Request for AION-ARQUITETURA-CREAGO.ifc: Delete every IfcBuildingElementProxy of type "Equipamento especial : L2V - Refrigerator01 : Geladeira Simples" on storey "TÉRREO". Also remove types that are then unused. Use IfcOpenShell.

First a look at what the model holds.

```python
import ifcopenshell
import ifcopenshell.util.element

model = ifcopenshell.open("AION-ARQUITETURA-CREAGO.ifc")
print(model.schema)
storey = next(s for s in model.by_type("IfcBuildingStorey") if s.Name == "TÉRREO")
proxies = [e for e in ifcopenshell.util.element.get_decomposition(storey) if e.is_a("IfcBuildingElementProxy")]
seen = {}
for e in proxies:
    element_type = ifcopenshell.util.element.get_type(e)
    name = element_type.Name if element_type not in (None, e) else None
    seen[name] = seen.get(name, 0) + 1
for name, count in sorted(seen.items(), key=str):
    print(count, "x", name)
```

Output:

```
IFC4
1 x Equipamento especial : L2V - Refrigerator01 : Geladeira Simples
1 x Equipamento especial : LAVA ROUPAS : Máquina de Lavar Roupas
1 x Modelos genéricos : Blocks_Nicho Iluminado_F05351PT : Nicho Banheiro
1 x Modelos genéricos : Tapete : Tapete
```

```python
import ifcopenshell
import ifcopenshell.api.root
import ifcopenshell.util.element

model = ifcopenshell.open("AION-ARQUITETURA-CREAGO.ifc")

storey = next(s for s in model.by_type("IfcBuildingStorey") if s.Name == "TÉRREO")
proxies = [e for e in ifcopenshell.util.element.get_decomposition(storey) if e.is_a("IfcBuildingElementProxy")]
targets = [e for e in proxies if (t := ifcopenshell.util.element.get_type(e)) not in (None, e) and t.Name == "Equipamento especial : L2V - Refrigerator01 : Geladeira Simples"]
types = {ifcopenshell.util.element.get_type(e) for e in targets} - {None, *targets}

for e in targets:
    ifcopenshell.api.root.remove_product(model, product=e)
print(len(targets), "removed")

unused = [t for t in types if not ifcopenshell.util.element.get_types(t)]
for t in unused:
    ifcopenshell.api.root.remove_product(model, product=t)
print(len(unused), "unused types removed")

model.write("AION-ARQUITETURA-CREAGO_rev.ifc")
```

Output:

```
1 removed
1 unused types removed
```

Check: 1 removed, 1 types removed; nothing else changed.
